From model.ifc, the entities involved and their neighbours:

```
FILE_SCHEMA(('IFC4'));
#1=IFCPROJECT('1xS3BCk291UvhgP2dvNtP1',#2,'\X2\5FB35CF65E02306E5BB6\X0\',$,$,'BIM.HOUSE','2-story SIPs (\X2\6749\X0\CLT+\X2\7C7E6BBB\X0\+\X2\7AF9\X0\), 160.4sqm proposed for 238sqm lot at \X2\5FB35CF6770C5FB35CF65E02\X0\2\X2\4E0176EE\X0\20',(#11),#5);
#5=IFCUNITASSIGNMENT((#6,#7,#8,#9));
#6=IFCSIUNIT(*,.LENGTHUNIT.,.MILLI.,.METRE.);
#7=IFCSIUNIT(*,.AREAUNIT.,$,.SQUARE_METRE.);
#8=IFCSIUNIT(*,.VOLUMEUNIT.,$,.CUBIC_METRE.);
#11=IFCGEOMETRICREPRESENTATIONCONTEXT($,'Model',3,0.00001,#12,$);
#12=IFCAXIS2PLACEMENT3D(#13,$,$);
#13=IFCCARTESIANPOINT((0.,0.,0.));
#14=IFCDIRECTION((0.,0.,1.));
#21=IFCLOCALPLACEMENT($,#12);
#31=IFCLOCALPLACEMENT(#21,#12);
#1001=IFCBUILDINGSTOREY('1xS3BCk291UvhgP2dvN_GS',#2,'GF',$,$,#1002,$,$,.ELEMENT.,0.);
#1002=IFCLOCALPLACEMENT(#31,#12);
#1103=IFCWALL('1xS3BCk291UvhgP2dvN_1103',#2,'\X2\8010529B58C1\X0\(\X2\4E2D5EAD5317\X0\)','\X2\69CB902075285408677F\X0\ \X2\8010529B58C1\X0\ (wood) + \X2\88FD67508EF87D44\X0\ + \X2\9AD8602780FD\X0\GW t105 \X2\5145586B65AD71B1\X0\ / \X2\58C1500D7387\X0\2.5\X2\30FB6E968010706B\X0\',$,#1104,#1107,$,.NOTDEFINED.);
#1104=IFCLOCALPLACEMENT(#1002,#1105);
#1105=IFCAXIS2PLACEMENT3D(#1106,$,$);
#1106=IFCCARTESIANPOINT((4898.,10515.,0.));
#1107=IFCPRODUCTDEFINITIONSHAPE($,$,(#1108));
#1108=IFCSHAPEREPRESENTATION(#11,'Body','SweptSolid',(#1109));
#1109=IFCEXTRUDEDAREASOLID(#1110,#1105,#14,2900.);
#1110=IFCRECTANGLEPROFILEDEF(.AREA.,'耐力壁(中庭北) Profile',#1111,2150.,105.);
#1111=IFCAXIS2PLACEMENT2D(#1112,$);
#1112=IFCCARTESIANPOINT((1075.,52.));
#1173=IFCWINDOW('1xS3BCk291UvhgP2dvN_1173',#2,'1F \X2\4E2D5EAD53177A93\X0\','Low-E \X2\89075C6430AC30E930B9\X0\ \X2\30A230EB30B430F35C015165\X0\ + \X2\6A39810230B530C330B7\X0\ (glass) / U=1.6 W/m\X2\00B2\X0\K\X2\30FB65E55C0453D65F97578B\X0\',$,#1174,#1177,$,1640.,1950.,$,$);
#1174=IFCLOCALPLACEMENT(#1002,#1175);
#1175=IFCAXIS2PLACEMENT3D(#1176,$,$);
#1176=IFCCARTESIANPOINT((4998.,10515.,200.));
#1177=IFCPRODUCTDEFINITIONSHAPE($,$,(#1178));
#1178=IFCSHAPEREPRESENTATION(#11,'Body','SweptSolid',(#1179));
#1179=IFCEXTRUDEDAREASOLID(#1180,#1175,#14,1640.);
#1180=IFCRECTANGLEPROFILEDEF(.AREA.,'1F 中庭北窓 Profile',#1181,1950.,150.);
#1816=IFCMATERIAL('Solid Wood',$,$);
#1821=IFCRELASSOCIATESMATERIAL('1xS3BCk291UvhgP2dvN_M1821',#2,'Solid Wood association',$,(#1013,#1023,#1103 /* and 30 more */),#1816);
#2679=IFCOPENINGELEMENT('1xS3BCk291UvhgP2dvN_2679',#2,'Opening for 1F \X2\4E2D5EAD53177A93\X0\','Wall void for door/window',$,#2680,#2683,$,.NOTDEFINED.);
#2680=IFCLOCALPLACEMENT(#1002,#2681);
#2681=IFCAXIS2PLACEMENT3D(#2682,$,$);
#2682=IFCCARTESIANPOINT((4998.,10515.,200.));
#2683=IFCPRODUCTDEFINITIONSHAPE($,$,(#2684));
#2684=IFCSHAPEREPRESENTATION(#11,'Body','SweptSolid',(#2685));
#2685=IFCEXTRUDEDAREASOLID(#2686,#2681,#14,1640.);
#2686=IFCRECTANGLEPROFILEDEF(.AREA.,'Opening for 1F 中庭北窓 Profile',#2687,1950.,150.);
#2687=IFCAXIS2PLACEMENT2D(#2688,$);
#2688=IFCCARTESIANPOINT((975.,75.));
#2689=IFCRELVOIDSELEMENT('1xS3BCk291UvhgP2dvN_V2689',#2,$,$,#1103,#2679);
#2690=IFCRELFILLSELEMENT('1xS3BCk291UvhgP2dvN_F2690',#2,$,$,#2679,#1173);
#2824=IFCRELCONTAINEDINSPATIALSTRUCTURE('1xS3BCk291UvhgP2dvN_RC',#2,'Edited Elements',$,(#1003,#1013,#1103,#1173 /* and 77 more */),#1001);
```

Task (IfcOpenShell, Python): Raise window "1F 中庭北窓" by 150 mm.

```python
import numpy as np
import ifcopenshell
import ifcopenshell.api.geometry
import ifcopenshell.util.placement
import ifcopenshell.util.unit

model = ifcopenshell.open("model.ifc")
unit_scale = ifcopenshell.util.unit.calculate_unit_scale(model)

window = model.by_id(1173)
opening = window.FillsVoids[0].RelatingOpeningElement
dz = 0.15 / unit_scale

shift = np.array([0.0, 0.0, dz])
# The window is not placed relative to its opening, so move both.
for product in (opening, window):
    matrix = ifcopenshell.util.placement.get_local_placement(product.ObjectPlacement)
    matrix[:3, 3] += shift
    ifcopenshell.api.geometry.edit_object_placement(model, product=product, matrix=matrix, is_si=False)

print(f"moved by {dz * unit_scale:+.3f} m")

model.write("model_updated.ifc")
```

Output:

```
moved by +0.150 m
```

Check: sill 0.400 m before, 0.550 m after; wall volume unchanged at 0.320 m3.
